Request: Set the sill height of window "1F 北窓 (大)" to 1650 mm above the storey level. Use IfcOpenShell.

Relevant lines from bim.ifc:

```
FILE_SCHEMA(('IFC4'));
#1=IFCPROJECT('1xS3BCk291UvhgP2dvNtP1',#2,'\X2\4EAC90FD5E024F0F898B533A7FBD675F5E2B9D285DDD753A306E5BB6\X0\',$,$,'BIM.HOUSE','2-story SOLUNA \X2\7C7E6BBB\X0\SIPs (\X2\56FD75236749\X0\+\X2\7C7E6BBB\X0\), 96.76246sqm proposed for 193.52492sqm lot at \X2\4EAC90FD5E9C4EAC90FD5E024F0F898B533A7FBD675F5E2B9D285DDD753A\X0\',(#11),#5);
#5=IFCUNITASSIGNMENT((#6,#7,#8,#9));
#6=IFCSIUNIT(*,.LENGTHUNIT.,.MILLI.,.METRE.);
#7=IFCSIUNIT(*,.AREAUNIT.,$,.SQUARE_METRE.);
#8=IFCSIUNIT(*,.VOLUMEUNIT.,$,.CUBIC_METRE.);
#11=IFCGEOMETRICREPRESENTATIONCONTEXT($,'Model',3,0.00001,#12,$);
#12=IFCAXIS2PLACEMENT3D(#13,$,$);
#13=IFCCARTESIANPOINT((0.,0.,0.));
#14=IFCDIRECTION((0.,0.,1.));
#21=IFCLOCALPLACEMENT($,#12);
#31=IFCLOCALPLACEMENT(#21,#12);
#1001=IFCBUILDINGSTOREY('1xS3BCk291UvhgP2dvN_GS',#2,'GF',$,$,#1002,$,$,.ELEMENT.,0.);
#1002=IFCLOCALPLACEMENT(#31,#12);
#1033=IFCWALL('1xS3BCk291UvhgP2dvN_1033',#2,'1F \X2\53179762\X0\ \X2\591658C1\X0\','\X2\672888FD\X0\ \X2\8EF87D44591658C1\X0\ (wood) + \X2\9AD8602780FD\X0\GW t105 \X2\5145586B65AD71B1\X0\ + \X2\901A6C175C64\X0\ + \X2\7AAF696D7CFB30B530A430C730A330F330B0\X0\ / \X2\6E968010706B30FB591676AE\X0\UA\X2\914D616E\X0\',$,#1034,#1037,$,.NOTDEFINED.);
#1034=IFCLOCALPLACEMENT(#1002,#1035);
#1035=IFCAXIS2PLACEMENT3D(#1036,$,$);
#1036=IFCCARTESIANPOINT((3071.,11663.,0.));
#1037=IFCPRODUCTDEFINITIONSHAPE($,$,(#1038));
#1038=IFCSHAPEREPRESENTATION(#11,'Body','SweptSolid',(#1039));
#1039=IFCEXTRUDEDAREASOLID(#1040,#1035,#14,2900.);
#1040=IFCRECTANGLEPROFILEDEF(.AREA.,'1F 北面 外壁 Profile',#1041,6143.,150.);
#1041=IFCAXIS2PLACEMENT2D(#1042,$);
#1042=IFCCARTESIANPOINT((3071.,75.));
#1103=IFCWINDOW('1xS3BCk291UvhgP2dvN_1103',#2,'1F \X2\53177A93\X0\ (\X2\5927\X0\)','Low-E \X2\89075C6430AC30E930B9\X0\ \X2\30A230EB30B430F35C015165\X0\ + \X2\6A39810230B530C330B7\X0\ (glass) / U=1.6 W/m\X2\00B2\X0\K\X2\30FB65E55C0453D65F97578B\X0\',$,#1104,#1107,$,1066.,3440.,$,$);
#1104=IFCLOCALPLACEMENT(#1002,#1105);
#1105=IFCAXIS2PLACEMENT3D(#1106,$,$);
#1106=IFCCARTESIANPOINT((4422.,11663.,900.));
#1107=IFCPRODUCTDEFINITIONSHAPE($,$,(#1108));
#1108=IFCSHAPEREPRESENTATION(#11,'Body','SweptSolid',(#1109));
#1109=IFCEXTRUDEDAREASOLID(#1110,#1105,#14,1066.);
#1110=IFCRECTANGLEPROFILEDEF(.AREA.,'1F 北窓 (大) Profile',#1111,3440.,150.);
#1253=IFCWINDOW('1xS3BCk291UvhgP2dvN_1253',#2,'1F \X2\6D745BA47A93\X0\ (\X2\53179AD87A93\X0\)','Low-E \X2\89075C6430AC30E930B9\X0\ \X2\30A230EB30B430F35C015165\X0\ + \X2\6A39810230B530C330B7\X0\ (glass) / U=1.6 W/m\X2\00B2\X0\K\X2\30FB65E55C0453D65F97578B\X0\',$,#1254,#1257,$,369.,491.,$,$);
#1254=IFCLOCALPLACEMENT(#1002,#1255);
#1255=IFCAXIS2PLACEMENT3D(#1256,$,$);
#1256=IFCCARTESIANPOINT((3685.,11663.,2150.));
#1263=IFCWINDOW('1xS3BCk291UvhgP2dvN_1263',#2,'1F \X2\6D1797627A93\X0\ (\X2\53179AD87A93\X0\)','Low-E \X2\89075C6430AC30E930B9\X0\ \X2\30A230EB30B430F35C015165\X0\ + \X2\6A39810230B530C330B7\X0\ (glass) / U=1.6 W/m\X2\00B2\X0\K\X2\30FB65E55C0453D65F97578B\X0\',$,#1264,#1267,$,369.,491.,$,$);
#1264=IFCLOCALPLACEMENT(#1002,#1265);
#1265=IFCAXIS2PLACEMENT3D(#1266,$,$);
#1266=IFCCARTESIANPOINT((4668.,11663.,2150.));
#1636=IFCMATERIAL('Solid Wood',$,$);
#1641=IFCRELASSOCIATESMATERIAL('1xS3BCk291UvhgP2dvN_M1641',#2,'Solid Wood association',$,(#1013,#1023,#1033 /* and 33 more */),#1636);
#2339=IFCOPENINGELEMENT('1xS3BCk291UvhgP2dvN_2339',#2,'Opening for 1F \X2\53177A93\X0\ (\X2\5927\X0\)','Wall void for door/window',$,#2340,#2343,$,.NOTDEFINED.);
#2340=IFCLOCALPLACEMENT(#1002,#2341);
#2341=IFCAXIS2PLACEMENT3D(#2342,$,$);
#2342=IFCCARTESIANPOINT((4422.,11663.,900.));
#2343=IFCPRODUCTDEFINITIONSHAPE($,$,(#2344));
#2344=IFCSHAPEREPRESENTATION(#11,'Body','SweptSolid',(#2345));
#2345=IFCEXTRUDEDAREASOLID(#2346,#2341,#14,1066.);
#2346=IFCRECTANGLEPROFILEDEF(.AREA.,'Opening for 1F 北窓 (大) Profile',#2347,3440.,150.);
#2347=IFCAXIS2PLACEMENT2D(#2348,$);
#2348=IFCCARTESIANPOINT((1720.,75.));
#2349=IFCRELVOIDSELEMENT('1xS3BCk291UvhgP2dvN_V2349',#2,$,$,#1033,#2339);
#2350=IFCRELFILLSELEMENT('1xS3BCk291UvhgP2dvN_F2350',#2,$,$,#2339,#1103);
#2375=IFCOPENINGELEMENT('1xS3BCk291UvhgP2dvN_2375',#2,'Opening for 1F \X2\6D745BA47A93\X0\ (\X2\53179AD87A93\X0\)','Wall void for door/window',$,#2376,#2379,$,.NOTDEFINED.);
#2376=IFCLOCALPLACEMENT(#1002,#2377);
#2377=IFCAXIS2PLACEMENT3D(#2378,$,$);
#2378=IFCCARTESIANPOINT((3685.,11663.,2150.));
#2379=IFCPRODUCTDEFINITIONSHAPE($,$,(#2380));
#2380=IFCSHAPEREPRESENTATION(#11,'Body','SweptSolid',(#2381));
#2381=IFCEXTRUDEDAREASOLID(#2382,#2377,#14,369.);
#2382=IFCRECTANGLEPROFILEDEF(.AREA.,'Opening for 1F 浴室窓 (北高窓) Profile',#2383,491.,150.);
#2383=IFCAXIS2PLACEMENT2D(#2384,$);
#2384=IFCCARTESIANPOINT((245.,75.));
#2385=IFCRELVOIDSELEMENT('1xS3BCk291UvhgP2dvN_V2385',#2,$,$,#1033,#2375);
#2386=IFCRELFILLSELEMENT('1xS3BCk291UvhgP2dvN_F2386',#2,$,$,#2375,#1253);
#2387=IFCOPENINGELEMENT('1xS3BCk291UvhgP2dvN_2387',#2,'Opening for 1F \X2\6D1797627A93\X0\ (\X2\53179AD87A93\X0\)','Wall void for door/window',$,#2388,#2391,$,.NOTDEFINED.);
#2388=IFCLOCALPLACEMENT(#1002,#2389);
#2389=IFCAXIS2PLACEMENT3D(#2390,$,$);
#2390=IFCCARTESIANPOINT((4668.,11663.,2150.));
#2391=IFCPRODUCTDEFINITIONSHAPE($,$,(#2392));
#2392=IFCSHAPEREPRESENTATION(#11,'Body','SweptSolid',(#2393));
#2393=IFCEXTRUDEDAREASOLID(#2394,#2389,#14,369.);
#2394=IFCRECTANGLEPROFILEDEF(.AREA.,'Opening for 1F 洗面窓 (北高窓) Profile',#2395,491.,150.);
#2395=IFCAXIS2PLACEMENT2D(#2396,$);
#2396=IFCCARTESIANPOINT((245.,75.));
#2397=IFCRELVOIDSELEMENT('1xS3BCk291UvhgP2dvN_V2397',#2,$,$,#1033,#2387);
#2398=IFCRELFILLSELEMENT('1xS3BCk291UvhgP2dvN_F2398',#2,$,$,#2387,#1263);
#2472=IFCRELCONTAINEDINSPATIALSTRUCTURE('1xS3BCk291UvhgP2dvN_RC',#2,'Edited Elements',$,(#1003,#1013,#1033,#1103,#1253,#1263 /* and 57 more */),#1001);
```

```python
import numpy as np
import ifcopenshell
import ifcopenshell.api.geometry
import ifcopenshell.geom
import ifcopenshell.util.element
import ifcopenshell.util.placement
import ifcopenshell.util.shape
import ifcopenshell.util.unit

model = ifcopenshell.open("bim.ifc")
unit_scale = ifcopenshell.util.unit.calculate_unit_scale(model)

window = model.by_id(1103)
opening = window.FillsVoids[0].RelatingOpeningElement
storey = ifcopenshell.util.element.get_container(window, ifc_class="IfcBuildingStorey")
level = ifcopenshell.util.placement.get_local_placement(storey.ObjectPlacement)[2, 3]

# The opening's origin need not be at the sill, so measure its lowest point.
shape = ifcopenshell.geom.create_shape(ifcopenshell.geom.settings(), opening)
bottom = ifcopenshell.util.shape.get_shape_bottom_elevation(shape, shape.geometry) / unit_scale
dz = level + 1650.0 - bottom

shift = np.array([0.0, 0.0, dz])
# The window is not placed relative to its opening, so move both.
for product in (opening, window):
    matrix = ifcopenshell.util.placement.get_local_placement(product.ObjectPlacement)
    matrix[:3, 3] += shift
    ifcopenshell.api.geometry.edit_object_placement(model, product=product, matrix=matrix, is_si=False)

print(f"moved by {dz * unit_scale:+.3f} m")

model.write("bim_rev.ifc")
```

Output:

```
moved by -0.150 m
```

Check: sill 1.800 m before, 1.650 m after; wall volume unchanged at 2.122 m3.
